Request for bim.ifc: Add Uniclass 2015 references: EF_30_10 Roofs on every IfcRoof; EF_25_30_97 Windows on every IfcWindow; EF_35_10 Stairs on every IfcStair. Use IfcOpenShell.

First a look at what the model holds.

```python
import ifcopenshell

model = ifcopenshell.open("bim.ifc")
print(model.schema)
print("classifications:", [c.Name for c in model.by_type("IfcClassification")])
for ifc_class in ("IfcDoor", "IfcRoof", "IfcStair", "IfcWall", "IfcWindow"):
    print(ifc_class, len(model.by_type(ifc_class)))
```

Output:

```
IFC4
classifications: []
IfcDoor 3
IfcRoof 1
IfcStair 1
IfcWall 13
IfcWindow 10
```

```python
import ifcopenshell
import ifcopenshell.api.classification

model = ifcopenshell.open("bim.ifc")

system = ifcopenshell.api.classification.add_classification(model, classification="Uniclass 2015")

codes = {
    "IfcRoof": ("EF_30_10", "Roofs"),
    "IfcWindow": ("EF_25_30_97", "Windows"),
    "IfcStair": ("EF_35_10", "Stairs"),
}
for ifc_class, (code, name) in codes.items():
    products = model.by_type(ifc_class)
    ifcopenshell.api.classification.add_reference(
        model, products=products, classification=system, identification=code, name=name
    )
    print(code, len(products))

model.write("bim_updated.ifc")
```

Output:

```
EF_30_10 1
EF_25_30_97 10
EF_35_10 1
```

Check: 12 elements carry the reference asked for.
